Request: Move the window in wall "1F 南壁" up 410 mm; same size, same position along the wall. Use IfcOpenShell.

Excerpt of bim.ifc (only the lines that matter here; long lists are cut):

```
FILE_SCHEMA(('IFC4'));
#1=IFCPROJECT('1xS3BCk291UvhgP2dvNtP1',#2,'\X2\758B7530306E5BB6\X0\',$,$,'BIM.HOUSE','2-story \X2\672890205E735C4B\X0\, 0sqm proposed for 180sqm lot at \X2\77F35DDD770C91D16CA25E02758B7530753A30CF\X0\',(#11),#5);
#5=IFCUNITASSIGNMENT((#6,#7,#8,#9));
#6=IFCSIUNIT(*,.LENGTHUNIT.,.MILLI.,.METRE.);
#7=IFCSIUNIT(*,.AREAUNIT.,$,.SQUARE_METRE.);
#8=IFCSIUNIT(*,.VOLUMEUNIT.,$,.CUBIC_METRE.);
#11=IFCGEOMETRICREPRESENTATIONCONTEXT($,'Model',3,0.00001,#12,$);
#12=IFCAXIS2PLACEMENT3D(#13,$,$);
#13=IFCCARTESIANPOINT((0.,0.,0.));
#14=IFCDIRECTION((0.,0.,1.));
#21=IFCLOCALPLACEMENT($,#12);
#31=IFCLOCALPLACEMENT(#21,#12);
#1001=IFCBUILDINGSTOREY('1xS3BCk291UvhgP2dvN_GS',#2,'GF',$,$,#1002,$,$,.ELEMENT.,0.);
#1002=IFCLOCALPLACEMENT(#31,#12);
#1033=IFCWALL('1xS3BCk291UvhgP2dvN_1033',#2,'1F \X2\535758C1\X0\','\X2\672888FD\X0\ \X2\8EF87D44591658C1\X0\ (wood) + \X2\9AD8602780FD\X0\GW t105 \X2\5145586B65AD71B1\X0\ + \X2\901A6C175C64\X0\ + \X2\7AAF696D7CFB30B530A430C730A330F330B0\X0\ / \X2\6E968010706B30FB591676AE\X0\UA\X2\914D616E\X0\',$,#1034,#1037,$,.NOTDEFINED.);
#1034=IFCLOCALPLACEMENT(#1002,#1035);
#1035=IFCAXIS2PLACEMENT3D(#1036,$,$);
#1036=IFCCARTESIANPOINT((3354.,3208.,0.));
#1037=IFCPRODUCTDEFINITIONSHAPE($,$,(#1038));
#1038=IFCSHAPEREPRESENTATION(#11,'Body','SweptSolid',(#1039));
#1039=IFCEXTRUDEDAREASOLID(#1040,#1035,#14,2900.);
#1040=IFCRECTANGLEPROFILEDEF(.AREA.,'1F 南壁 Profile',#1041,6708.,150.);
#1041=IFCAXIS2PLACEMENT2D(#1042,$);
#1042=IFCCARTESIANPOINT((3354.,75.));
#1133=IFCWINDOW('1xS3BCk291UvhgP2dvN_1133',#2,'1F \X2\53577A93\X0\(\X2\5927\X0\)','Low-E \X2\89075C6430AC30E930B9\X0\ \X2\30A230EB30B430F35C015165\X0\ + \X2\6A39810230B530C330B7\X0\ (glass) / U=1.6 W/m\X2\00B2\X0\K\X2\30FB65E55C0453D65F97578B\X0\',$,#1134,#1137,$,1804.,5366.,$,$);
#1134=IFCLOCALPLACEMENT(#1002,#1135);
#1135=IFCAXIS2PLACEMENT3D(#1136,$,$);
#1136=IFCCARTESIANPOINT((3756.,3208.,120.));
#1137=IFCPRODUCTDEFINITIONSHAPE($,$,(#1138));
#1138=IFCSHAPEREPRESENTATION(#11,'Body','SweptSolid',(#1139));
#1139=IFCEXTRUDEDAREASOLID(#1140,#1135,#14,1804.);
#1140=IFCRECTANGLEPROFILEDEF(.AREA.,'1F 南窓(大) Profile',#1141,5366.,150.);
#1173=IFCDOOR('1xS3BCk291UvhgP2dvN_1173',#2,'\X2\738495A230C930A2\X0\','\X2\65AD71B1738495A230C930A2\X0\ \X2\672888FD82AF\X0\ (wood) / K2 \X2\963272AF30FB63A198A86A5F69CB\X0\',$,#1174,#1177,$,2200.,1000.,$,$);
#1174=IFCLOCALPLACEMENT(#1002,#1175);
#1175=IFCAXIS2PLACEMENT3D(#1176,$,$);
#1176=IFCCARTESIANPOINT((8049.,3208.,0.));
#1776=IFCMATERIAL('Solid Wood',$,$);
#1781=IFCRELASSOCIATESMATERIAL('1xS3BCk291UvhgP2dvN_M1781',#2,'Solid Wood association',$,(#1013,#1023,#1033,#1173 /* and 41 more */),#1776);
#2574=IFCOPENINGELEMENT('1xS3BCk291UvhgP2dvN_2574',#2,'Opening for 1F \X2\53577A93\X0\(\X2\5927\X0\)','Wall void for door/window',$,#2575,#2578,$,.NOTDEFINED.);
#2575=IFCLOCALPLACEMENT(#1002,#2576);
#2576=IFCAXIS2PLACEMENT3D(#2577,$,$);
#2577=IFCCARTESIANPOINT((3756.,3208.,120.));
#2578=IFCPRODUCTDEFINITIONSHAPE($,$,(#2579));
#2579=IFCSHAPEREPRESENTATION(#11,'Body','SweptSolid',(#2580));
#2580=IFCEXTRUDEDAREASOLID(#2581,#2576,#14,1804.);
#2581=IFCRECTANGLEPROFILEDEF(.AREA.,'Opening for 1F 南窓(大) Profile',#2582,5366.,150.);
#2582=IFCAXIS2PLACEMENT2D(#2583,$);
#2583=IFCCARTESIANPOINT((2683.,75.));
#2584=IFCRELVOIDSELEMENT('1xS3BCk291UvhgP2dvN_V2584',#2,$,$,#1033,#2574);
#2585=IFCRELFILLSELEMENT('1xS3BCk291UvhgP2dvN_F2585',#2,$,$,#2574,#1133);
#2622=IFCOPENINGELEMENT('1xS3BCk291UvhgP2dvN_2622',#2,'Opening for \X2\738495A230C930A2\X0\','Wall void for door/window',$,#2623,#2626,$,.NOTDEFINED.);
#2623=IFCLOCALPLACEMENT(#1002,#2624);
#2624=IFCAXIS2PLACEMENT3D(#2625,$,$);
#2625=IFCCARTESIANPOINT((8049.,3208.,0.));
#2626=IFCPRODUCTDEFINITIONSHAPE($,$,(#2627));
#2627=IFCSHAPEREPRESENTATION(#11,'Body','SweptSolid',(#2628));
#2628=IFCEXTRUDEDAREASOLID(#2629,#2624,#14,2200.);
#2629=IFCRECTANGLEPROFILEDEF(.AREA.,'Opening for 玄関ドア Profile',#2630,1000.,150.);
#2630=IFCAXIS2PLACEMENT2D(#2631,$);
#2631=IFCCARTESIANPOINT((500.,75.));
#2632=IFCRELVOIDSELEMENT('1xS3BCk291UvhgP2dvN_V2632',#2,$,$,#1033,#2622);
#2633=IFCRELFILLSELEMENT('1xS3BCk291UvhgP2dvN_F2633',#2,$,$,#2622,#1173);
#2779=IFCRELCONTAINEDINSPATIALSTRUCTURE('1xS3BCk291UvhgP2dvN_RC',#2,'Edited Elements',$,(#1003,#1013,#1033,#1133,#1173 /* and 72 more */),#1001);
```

```python
import numpy as np
import ifcopenshell
import ifcopenshell.api.geometry
import ifcopenshell.util.placement
import ifcopenshell.util.unit

model = ifcopenshell.open("bim.ifc")
unit_scale = ifcopenshell.util.unit.calculate_unit_scale(model)

window = model.by_guid("1xS3BCk291UvhgP2dvN_1133")
opening = window.FillsVoids[0].RelatingOpeningElement
dz = 410.0

shift = np.array([0.0, 0.0, dz])
# The window is not placed relative to its opening, so move both.
for product in (opening, window):
    matrix = ifcopenshell.util.placement.get_local_placement(product.ObjectPlacement)
    matrix[:3, 3] += shift
    ifcopenshell.api.geometry.edit_object_placement(model, product=product, matrix=matrix, is_si=False)

print(f"moved by {dz * unit_scale:+.3f} m")

model.write("bim_edited.ifc")
```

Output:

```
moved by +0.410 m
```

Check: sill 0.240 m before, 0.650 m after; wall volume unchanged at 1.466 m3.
